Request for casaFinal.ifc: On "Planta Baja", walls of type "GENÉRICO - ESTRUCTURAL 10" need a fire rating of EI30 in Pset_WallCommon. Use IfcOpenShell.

First a look at what the model holds.

```python
import ifcopenshell
import ifcopenshell.util.element

model = ifcopenshell.open("casaFinal.ifc")
print(model.schema)
storey = next(s for s in model.by_type("IfcBuildingStorey") if s.Name == "Planta Baja")
walls = [e for e in ifcopenshell.util.element.get_decomposition(storey) if e.is_a("IfcWall")]
seen = {}
for e in walls:
    element_type = ifcopenshell.util.element.get_type(e)
    key = (element_type.Name if element_type != e and element_type else None, ifcopenshell.util.element.get_pset(e, "Pset_WallCommon", "FireRating"))
    seen[key] = seen.get(key, 0) + 1
for (name, value), count in sorted(seen.items(), key=str):
    print(count, "x", name, "|", value)
```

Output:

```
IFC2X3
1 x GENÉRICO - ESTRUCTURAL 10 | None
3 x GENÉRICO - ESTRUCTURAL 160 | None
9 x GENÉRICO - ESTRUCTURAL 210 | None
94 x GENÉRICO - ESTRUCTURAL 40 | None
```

```python
import ifcopenshell
import ifcopenshell.api.pset
import ifcopenshell.util.element

model = ifcopenshell.open("casaFinal.ifc")

storey = next(s for s in model.by_type("IfcBuildingStorey") if s.Name == "Planta Baja")
walls = [e for e in ifcopenshell.util.element.get_decomposition(storey) if e.is_a("IfcWall")]

count = 0
for e in walls:
    element_type = ifcopenshell.util.element.get_type(e)
    if element_type in (None, e) or element_type.Name != "GENÉRICO - ESTRUCTURAL 10":
        continue
    # add_pset returns the element's existing set when there is one.
    pset = ifcopenshell.api.pset.add_pset(model, product=e, name="Pset_WallCommon")
    ifcopenshell.api.pset.edit_pset(model, pset=pset, properties={"FireRating": "EI30"})
    count += 1

print(count, "walls updated")

model.write("casaFinal_edited.ifc")
```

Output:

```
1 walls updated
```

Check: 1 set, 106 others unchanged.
